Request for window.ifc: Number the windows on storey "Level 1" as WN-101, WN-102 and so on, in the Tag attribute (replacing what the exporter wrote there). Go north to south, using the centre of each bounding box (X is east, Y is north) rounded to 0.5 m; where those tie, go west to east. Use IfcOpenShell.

First a look at what the model holds.

```python
import ifcopenshell
import ifcopenshell.util.element
import ifcopenshell.util.placement

model = ifcopenshell.open("window.ifc")
print(model.schema)
storey = next(s for s in model.by_type("IfcBuildingStorey") if s.Name == "Level 1")
windows = [e for e in ifcopenshell.util.element.get_decomposition(storey) if e.is_a("IfcWindow")]
for e in sorted(windows, key=lambda e: e.id()):
    origin = ifcopenshell.util.placement.get_local_placement(e.ObjectPlacement)[:3, 3]
    print(e.id(), e.Tag, e.Name, origin.round(2) + 0.0, sep=" | ")
```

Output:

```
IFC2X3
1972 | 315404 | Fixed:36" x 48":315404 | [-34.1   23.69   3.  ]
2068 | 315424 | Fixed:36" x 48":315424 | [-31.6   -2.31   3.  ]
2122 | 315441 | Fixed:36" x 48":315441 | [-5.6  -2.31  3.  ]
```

```python
import ifcopenshell
import ifcopenshell.geom
import ifcopenshell.util.element
import ifcopenshell.util.shape

model = ifcopenshell.open("window.ifc")
settings = ifcopenshell.geom.settings()
settings.set("use-world-coords", True)


def centre(element):
    shape = ifcopenshell.geom.create_shape(settings, element)
    return ifcopenshell.util.shape.get_bbox_centroid(shape.geometry)


storey = next(s for s in model.by_type("IfcBuildingStorey") if s.Name == "Level 1")
windows = [e for e in ifcopenshell.util.element.get_decomposition(storey) if e.is_a("IfcWindow")]

# Insertion points can sit at a corner or the storey origin, so sort by the geometry (in metres).
centres = {e: centre(e) for e in windows}
windows.sort(key=lambda e: (-round(centres[e][1] / 0.5), centres[e][0]))

for i, e in enumerate(windows, start=1):
    number = f"WN-1{i:02d}"
    e.Tag = number
    print(e.id(), number)

model.write("window_updated.ifc")
```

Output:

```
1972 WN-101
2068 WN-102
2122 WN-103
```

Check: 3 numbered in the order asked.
